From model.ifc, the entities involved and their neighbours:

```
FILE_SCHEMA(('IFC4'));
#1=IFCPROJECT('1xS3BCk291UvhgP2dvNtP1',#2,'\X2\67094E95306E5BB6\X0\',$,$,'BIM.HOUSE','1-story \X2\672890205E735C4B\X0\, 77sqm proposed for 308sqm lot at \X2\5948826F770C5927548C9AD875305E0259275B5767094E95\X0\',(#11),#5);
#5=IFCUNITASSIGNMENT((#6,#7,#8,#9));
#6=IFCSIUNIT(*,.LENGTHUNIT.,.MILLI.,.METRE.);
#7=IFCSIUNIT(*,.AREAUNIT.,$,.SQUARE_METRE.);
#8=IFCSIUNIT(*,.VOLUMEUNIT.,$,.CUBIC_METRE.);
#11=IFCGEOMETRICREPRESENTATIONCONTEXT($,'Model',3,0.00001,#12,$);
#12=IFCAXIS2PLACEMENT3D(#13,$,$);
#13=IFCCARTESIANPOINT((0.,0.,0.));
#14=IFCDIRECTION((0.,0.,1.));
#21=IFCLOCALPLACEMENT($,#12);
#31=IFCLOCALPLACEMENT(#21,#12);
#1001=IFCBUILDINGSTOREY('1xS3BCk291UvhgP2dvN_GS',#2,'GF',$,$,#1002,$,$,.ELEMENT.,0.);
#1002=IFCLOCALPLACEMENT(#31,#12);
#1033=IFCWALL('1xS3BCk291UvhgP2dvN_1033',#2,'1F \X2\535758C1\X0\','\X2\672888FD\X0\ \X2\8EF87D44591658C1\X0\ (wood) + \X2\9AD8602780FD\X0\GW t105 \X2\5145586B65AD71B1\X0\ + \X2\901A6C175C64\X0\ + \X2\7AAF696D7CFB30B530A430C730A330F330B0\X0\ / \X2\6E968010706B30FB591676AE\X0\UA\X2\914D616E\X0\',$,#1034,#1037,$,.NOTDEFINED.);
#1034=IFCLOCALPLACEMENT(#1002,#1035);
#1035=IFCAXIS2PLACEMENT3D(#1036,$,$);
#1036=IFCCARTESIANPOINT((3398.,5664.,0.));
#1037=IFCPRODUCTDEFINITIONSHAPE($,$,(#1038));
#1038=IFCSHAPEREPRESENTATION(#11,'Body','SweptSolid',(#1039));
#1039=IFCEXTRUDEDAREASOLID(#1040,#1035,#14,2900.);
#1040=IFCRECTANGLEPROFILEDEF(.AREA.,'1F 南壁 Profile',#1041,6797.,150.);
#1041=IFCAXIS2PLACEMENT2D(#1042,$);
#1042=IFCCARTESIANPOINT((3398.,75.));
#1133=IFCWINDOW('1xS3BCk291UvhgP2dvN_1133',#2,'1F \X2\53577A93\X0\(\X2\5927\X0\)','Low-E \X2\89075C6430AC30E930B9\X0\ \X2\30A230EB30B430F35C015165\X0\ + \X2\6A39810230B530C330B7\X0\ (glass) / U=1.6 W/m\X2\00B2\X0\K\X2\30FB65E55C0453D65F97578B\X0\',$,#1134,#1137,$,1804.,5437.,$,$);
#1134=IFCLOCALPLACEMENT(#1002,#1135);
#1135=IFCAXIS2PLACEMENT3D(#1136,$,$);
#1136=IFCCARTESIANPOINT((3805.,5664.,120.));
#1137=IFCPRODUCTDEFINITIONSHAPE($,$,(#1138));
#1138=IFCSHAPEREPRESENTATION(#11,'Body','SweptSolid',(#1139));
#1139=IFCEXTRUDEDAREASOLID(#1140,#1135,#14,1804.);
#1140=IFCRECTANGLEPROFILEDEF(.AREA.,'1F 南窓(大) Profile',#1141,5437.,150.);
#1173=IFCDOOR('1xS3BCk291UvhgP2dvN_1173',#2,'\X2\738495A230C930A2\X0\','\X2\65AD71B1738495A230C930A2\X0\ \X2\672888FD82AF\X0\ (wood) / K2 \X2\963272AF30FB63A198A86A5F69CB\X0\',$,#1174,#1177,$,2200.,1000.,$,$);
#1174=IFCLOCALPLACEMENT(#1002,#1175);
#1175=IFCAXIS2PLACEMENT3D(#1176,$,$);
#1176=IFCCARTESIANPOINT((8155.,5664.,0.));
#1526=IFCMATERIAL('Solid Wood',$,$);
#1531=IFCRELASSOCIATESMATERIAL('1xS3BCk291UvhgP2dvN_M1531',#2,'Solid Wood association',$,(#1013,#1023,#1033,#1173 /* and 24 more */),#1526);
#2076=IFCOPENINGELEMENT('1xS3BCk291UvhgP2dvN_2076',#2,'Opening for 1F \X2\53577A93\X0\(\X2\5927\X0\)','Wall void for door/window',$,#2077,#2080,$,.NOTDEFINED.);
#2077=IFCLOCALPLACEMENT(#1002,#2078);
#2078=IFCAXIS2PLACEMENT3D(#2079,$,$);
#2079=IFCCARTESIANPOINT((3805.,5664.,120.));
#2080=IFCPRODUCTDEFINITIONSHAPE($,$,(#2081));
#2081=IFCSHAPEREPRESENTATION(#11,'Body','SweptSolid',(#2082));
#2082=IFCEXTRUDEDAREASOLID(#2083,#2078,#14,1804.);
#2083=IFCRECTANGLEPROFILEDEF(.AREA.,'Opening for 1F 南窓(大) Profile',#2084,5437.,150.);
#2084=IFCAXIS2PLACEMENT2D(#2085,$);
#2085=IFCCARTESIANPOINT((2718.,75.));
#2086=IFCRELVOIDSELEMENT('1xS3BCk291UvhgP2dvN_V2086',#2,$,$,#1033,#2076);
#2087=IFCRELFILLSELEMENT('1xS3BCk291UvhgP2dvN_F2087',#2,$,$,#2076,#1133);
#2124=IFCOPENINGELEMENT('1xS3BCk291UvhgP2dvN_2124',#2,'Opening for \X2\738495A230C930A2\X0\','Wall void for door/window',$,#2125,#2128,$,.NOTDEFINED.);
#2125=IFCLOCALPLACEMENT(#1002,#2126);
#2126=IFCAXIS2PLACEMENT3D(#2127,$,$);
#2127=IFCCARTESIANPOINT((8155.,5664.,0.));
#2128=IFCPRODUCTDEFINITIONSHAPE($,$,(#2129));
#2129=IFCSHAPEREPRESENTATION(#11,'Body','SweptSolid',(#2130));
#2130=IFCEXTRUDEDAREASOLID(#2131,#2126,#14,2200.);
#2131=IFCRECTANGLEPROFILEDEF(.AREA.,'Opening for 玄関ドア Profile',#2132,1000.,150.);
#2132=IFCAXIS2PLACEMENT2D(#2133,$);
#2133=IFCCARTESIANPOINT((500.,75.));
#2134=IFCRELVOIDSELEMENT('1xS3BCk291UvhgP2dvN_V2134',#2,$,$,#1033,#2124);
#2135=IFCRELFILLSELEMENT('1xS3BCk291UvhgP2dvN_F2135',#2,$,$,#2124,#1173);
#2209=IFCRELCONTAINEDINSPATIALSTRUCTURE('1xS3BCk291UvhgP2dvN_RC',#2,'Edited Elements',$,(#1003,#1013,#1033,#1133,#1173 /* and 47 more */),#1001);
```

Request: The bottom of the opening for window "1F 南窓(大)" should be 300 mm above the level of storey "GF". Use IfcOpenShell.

```python
import numpy as np
import ifcopenshell
import ifcopenshell.api.geometry
import ifcopenshell.geom
import ifcopenshell.util.element
import ifcopenshell.util.placement
import ifcopenshell.util.shape
import ifcopenshell.util.unit

model = ifcopenshell.open("model.ifc")
unit_scale = ifcopenshell.util.unit.calculate_unit_scale(model)

window = model.by_id(1133)
opening = window.FillsVoids[0].RelatingOpeningElement
storey = ifcopenshell.util.element.get_container(window, ifc_class="IfcBuildingStorey")
level = ifcopenshell.util.placement.get_local_placement(storey.ObjectPlacement)[2, 3]

# The opening's origin need not be at the sill, so measure its lowest point.
shape = ifcopenshell.geom.create_shape(ifcopenshell.geom.settings(), opening)
bottom = ifcopenshell.util.shape.get_shape_bottom_elevation(shape, shape.geometry) / unit_scale
dz = level + 300.0 - bottom

shift = np.array([0.0, 0.0, dz])
# The window is not placed relative to its opening, so move both.
for product in (opening, window):
    matrix = ifcopenshell.util.placement.get_local_placement(product.ObjectPlacement)
    matrix[:3, 3] += shift
    ifcopenshell.api.geometry.edit_object_placement(model, product=product, matrix=matrix, is_si=False)

print(f"moved by {dz * unit_scale:+.3f} m")

model.write("model_rev.ifc")
```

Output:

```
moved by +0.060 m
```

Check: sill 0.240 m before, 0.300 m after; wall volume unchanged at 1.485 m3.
